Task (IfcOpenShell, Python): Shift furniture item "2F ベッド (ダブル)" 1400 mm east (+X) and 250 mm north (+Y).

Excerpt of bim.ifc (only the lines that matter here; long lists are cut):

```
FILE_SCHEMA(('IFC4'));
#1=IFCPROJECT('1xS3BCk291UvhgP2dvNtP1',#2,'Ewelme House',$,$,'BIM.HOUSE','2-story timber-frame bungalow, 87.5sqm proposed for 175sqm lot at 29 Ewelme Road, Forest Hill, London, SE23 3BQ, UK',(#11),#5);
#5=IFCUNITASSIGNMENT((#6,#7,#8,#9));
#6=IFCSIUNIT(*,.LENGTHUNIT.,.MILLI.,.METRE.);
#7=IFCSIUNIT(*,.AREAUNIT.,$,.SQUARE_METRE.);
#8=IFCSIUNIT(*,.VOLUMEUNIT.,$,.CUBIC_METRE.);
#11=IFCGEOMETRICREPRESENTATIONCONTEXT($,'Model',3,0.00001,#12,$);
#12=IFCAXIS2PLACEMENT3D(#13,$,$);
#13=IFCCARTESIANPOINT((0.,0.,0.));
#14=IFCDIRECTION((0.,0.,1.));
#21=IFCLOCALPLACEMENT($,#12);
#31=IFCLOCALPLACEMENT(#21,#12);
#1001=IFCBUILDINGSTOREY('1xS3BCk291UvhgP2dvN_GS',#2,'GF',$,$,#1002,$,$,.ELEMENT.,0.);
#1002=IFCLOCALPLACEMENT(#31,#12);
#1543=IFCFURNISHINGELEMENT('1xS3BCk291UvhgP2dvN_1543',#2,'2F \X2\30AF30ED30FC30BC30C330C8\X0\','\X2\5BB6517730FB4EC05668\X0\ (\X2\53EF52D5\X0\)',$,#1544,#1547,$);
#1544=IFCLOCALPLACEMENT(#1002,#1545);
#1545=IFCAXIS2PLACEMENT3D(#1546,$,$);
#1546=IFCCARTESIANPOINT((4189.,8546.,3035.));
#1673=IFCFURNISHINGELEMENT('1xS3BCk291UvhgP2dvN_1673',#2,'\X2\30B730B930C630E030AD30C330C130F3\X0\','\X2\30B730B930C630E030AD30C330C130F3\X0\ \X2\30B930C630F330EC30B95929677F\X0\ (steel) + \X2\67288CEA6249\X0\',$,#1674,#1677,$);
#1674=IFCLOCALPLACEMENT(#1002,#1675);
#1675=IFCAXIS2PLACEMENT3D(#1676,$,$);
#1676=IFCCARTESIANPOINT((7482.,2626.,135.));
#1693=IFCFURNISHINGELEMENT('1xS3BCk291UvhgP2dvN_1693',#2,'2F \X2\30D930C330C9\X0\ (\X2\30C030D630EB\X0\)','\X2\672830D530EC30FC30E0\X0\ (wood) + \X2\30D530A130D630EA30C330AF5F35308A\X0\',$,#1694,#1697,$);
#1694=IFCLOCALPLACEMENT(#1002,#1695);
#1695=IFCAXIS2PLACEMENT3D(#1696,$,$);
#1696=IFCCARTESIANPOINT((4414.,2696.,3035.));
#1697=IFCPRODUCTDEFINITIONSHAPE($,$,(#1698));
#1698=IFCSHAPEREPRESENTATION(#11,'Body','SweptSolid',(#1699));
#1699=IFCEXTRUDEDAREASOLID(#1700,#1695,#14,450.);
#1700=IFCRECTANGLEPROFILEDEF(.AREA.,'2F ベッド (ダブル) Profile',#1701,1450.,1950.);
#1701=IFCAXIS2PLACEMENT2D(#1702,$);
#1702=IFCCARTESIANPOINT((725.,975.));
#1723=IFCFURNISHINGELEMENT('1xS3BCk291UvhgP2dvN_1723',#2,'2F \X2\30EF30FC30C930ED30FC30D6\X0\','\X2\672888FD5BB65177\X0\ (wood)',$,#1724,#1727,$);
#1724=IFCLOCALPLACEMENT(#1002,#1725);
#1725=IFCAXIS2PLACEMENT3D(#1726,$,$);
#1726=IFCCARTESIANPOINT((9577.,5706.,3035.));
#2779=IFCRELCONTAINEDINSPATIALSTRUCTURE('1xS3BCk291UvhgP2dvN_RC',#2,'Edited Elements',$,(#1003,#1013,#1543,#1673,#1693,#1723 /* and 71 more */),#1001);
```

```python
import ifcopenshell
import ifcopenshell.api.geometry
import ifcopenshell.util.placement

model = ifcopenshell.open("bim.ifc")

item = model.by_id(1693)
matrix = ifcopenshell.util.placement.get_local_placement(item.ObjectPlacement)
matrix[0, 3] += 1400.0
matrix[1, 3] += 250.0
ifcopenshell.api.geometry.edit_object_placement(model, product=item, matrix=matrix, is_si=False)

print(ifcopenshell.util.placement.get_local_placement(item.ObjectPlacement).round(3) + 0.0)

model.write("bim_edited.ifc")
```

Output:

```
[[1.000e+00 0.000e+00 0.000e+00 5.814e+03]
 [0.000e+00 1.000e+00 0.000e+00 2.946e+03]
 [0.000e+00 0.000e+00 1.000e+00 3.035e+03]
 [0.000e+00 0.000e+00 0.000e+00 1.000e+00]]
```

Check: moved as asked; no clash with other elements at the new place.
